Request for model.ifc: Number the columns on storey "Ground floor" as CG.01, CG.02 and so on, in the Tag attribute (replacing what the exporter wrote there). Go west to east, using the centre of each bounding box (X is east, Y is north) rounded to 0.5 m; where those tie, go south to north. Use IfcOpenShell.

First a look at what the model holds.

```python
import ifcopenshell
import ifcopenshell.util.element
import ifcopenshell.util.placement

model = ifcopenshell.open("model.ifc")
print(model.schema)
storey = next(s for s in model.by_type("IfcBuildingStorey") if s.Name == "Ground floor")
columns = [e for e in ifcopenshell.util.element.get_decomposition(storey) if e.is_a("IfcColumn")]
for e in sorted(columns, key=lambda e: e.id()):
    origin = ifcopenshell.util.placement.get_local_placement(e.ObjectPlacement)[:3, 3]
    print(e.id(), e.Tag, e.Name, origin.round(2) + 0.0, sep=" | ")
```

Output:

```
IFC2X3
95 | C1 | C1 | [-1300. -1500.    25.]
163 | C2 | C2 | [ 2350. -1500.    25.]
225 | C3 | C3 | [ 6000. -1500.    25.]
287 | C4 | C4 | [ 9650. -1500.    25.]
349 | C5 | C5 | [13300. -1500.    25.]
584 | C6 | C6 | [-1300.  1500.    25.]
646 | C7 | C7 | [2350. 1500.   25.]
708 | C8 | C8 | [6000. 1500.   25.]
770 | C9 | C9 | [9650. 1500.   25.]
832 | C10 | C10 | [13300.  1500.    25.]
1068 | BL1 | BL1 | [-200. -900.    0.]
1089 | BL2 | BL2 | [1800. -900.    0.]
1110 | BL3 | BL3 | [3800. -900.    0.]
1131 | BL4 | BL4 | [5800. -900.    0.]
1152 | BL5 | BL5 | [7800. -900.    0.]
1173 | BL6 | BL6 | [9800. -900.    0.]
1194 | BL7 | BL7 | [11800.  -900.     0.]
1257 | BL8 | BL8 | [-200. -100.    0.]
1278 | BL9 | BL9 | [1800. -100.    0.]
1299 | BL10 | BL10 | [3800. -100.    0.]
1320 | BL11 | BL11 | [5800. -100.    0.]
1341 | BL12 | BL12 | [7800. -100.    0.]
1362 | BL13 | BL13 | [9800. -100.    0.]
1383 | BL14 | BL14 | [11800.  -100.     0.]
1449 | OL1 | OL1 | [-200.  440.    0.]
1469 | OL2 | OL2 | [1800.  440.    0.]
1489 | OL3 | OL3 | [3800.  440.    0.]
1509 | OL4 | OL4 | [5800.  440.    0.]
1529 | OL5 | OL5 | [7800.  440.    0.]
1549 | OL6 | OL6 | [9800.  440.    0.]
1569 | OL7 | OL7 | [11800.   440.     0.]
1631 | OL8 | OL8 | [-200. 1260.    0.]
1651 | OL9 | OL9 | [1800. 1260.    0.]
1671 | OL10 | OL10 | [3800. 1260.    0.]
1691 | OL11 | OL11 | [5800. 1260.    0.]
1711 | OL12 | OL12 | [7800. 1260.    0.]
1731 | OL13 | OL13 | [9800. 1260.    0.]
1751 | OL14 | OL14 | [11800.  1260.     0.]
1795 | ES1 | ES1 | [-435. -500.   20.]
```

```python
import ifcopenshell
import ifcopenshell.geom
import ifcopenshell.util.element
import ifcopenshell.util.shape

model = ifcopenshell.open("model.ifc")
settings = ifcopenshell.geom.settings()
settings.set("use-world-coords", True)


def centre(element):
    shape = ifcopenshell.geom.create_shape(settings, element)
    return ifcopenshell.util.shape.get_bbox_centroid(shape.geometry)


storey = next(s for s in model.by_type("IfcBuildingStorey") if s.Name == "Ground floor")
columns = [e for e in ifcopenshell.util.element.get_decomposition(storey) if e.is_a("IfcColumn")]

# Insertion points can sit at a corner or the storey origin, so sort by the geometry (in metres).
centres = {e: centre(e) for e in columns}
columns.sort(key=lambda e: (round(centres[e][0] / 0.5), centres[e][1]))

for i, e in enumerate(columns, start=1):
    number = f"CG.{i:02d}"
    e.Tag = number
    print(e.id(), number)

model.write("model-out.ifc")
```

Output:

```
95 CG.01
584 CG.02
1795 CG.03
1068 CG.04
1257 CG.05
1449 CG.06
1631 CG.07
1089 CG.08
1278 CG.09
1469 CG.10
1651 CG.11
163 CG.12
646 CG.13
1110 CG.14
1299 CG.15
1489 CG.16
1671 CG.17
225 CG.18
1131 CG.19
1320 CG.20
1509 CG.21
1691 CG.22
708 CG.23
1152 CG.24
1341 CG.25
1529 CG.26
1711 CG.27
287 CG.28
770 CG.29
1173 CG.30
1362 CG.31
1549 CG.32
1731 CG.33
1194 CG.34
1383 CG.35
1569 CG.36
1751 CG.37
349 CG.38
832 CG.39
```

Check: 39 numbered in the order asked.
